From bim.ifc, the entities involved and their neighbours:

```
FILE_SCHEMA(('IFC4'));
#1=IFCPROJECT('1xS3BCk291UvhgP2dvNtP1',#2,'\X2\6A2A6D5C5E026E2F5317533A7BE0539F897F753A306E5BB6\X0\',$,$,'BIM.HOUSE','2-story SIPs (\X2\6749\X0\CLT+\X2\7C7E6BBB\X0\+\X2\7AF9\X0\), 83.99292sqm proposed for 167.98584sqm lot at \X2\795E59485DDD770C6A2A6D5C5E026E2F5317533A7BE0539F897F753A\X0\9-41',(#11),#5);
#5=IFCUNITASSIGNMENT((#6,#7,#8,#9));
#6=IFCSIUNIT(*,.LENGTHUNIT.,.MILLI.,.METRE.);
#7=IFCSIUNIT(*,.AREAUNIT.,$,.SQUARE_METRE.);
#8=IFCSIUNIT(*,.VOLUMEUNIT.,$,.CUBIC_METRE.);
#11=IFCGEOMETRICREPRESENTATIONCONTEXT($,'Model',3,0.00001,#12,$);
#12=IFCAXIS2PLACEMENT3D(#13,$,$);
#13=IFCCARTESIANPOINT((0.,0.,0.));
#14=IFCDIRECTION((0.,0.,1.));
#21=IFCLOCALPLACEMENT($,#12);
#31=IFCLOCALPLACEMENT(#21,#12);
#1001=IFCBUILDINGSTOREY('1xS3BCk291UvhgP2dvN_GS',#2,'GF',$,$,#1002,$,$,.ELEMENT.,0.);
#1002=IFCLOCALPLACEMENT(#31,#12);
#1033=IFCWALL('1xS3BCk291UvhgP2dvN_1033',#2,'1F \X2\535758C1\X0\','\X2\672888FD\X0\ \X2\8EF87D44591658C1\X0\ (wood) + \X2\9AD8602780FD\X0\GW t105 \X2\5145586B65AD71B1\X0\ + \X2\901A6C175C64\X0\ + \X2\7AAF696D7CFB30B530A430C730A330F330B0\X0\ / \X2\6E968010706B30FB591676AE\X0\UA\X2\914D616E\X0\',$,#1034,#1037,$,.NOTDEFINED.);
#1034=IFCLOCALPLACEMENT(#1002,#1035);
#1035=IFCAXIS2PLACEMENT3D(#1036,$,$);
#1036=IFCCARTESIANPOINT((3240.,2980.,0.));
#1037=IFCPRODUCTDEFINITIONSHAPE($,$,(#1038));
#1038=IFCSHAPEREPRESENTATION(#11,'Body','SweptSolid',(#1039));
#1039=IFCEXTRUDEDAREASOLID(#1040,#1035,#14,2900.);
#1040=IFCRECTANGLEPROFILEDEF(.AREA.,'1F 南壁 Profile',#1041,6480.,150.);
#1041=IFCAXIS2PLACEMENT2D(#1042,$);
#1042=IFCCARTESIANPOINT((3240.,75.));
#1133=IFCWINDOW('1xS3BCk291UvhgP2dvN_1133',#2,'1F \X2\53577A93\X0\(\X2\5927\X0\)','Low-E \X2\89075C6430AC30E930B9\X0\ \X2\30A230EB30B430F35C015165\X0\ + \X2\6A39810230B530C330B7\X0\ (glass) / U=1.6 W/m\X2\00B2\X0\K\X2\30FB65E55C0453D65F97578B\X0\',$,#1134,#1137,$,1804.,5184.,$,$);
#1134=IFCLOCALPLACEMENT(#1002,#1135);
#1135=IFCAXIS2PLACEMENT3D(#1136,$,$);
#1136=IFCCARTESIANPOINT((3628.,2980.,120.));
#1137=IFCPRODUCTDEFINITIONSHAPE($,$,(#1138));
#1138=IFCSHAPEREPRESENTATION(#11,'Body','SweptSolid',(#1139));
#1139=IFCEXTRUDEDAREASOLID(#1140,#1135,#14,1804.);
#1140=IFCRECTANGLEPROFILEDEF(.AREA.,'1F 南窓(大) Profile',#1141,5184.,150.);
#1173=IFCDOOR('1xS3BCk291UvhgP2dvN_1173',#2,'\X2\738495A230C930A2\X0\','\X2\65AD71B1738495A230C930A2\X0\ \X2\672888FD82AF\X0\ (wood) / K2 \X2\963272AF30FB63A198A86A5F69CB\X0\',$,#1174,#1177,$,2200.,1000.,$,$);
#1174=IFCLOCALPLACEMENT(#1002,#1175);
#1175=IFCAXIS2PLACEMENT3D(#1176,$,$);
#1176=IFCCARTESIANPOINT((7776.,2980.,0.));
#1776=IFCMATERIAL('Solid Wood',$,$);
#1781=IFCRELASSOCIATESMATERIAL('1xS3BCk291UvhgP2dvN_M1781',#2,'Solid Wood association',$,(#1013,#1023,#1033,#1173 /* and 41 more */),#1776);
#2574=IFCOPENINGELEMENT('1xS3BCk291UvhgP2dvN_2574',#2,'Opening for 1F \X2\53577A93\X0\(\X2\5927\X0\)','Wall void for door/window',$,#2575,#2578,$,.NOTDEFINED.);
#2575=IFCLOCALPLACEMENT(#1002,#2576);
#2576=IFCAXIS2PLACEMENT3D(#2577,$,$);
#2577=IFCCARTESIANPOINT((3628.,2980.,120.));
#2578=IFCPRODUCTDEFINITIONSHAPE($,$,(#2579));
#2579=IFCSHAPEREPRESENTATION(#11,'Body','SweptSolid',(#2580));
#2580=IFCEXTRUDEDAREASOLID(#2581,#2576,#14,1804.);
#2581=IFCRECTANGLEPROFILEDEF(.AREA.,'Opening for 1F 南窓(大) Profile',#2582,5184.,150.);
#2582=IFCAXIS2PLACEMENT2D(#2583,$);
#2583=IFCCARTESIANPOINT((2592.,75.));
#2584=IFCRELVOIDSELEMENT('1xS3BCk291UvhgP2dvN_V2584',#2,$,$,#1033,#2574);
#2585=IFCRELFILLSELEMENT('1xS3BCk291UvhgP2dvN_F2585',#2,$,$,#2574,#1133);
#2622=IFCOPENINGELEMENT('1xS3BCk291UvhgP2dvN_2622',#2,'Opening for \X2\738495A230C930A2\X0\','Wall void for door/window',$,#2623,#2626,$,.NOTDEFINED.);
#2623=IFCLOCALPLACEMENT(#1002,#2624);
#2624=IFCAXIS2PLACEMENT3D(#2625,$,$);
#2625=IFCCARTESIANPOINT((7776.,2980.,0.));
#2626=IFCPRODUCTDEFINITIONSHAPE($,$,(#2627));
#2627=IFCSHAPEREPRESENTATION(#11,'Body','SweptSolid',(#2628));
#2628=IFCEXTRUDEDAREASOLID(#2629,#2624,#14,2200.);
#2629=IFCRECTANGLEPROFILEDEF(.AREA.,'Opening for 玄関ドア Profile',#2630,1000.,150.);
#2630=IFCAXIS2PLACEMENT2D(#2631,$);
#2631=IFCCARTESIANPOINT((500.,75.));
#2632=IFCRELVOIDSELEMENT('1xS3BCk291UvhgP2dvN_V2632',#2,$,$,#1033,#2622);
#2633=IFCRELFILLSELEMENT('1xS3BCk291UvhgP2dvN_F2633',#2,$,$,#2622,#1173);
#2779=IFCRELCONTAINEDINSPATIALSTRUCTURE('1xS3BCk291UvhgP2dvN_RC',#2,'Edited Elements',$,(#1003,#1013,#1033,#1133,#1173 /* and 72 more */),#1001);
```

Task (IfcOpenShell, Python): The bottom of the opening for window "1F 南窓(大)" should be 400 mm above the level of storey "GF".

```python
import numpy as np
import ifcopenshell
import ifcopenshell.api.geometry
import ifcopenshell.geom
import ifcopenshell.util.element
import ifcopenshell.util.placement
import ifcopenshell.util.shape
import ifcopenshell.util.unit

model = ifcopenshell.open("bim.ifc")
unit_scale = ifcopenshell.util.unit.calculate_unit_scale(model)

window = model.by_id(1133)
opening = window.FillsVoids[0].RelatingOpeningElement
storey = ifcopenshell.util.element.get_container(window, ifc_class="IfcBuildingStorey")
level = ifcopenshell.util.placement.get_local_placement(storey.ObjectPlacement)[2, 3]

# The opening's origin need not be at the sill, so measure its lowest point.
shape = ifcopenshell.geom.create_shape(ifcopenshell.geom.settings(), opening)
bottom = ifcopenshell.util.shape.get_shape_bottom_elevation(shape, shape.geometry) / unit_scale
dz = level + 0.4 / unit_scale - bottom

shift = np.array([0.0, 0.0, dz])
# The window is not placed relative to its opening, so move both.
for product in (opening, window):
    matrix = ifcopenshell.util.placement.get_local_placement(product.ObjectPlacement)
    matrix[:3, 3] += shift
    ifcopenshell.api.geometry.edit_object_placement(model, product=product, matrix=matrix, is_si=False)

print(f"moved by {dz * unit_scale:+.3f} m")

model.write("bim_edited.ifc")
```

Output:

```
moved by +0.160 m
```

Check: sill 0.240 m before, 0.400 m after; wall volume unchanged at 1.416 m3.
